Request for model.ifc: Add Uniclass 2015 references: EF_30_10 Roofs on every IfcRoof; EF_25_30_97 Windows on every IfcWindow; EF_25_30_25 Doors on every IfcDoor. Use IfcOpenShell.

First a look at what the model holds.

```python
import ifcopenshell

model = ifcopenshell.open("model.ifc")
print(model.schema)
print("classifications:", [c.Name for c in model.by_type("IfcClassification")])
for ifc_class in ("IfcDoor", "IfcRoof", "IfcStair", "IfcWall", "IfcWindow"):
    print(ifc_class, len(model.by_type(ifc_class)))
```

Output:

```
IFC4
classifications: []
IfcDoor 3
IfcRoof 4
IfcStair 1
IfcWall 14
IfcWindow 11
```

```python
import ifcopenshell
import ifcopenshell.api.classification

model = ifcopenshell.open("model.ifc")

system = ifcopenshell.api.classification.add_classification(model, classification="Uniclass 2015")

codes = {
    "IfcRoof": ("EF_30_10", "Roofs"),
    "IfcWindow": ("EF_25_30_97", "Windows"),
    "IfcDoor": ("EF_25_30_25", "Doors"),
}
for ifc_class, (code, name) in codes.items():
    products = model.by_type(ifc_class)
    ifcopenshell.api.classification.add_reference(
        model, products=products, classification=system, identification=code, name=name
    )
    print(code, len(products))

model.write("model_v2.ifc")
```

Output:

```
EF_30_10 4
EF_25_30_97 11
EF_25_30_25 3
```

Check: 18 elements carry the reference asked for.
